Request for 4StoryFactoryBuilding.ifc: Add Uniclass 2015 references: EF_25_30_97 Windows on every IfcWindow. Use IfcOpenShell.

First a look at what the model holds.

```python
import ifcopenshell

model = ifcopenshell.open("4StoryFactoryBuilding.ifc")
print(model.schema)
print("classifications:", [c.Name for c in model.by_type("IfcClassification")])
for ifc_class in ("IfcDoor", "IfcRoof", "IfcStair", "IfcWall", "IfcWindow"):
    print(ifc_class, len(model.by_type(ifc_class)))
```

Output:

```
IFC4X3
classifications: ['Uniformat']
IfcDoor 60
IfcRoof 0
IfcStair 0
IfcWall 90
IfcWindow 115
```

```python
import ifcopenshell
import ifcopenshell.api.classification

model = ifcopenshell.open("4StoryFactoryBuilding.ifc")

system = ifcopenshell.api.classification.add_classification(model, classification="Uniclass 2015")

codes = {
    "IfcWindow": ("EF_25_30_97", "Windows"),
}
for ifc_class, (code, name) in codes.items():
    products = model.by_type(ifc_class)
    ifcopenshell.api.classification.add_reference(
        model, products=products, classification=system, identification=code, name=name
    )
    print(code, len(products))

model.write("4StoryFactoryBuilding_edited.ifc")
```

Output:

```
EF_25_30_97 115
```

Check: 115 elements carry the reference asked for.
